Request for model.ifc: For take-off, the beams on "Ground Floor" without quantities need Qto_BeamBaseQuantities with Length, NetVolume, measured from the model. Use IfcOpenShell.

First a look at what the model holds.

```python
import ifcopenshell
import ifcopenshell.util.element
import ifcopenshell.util.unit

model = ifcopenshell.open("model.ifc")
print(model.schema)
for unit_type in ("LENGTHUNIT", "AREAUNIT", "VOLUMEUNIT"):
    print(unit_type, ifcopenshell.util.unit.calculate_unit_scale(model, unit_type))
storey = next(s for s in model.by_type("IfcBuildingStorey") if s.Name == "Ground Floor")
beams = [e for e in ifcopenshell.util.element.get_decomposition(storey) if e.is_a("IfcBeam")]
for e in sorted(beams, key=lambda e: e.id()):
    print(e.id(), e.is_a(), e.Name, list(ifcopenshell.util.element.get_psets(e, qtos_only=True)), sep=" | ")
```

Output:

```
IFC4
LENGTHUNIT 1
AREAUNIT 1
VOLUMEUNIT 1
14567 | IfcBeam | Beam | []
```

```python
import ifcopenshell
import ifcopenshell.api.pset
import ifcopenshell.geom
import ifcopenshell.util.element
import ifcopenshell.util.shape
import ifcopenshell.util.unit

model = ifcopenshell.open("model.ifc")
unit_scale = ifcopenshell.util.unit.calculate_unit_scale(model)
volume_scale = ifcopenshell.util.unit.calculate_unit_scale(model, "VOLUMEUNIT")
settings = ifcopenshell.geom.settings()

storey = next(s for s in model.by_type("IfcBuildingStorey") if s.Name == "Ground Floor")
beams = [e for e in ifcopenshell.util.element.get_decomposition(storey) if e.is_a("IfcBeam")]

for e in sorted(beams, key=lambda e: e.id()):
    if ifcopenshell.util.element.get_psets(e, qtos_only=True, should_inherit=False):
        continue
    # Geometry comes back in metres, in the element's own axes.
    shape = ifcopenshell.geom.create_shape(settings, e)
    values = {
        "Length": ifcopenshell.util.shape.get_max_xyz(shape.geometry) / unit_scale,
        "NetVolume": ifcopenshell.util.shape.get_volume(shape.geometry) / volume_scale,
    }
    qto = ifcopenshell.api.pset.add_qto(model, product=e, name="Qto_BeamBaseQuantities")
    ifcopenshell.api.pset.edit_qto(model, qto=qto, properties=values)
    print(e.id(), {k: round(v, 3) for k, v in values.items()})

model.write("model_v2.ifc")
```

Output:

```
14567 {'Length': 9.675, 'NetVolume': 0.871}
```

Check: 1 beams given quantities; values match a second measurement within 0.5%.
